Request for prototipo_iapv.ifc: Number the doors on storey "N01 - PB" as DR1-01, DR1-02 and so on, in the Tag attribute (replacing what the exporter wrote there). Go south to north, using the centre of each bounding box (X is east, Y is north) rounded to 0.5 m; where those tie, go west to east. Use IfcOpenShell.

First a look at what the model holds.

```python
import ifcopenshell
import ifcopenshell.util.element
import ifcopenshell.util.placement

model = ifcopenshell.open("prototipo_iapv.ifc")
print(model.schema)
storey = next(s for s in model.by_type("IfcBuildingStorey") if s.Name == "N01 - PB")
doors = [e for e in ifcopenshell.util.element.get_decomposition(storey) if e.is_a("IfcDoor")]
for e in sorted(doors, key=lambda e: e.id()):
    origin = ifcopenshell.util.placement.get_local_placement(e.ObjectPlacement)[:3, 3]
    print(e.id(), e.Tag, e.Name, origin.round(2) + 0.0, sep=" | ")
```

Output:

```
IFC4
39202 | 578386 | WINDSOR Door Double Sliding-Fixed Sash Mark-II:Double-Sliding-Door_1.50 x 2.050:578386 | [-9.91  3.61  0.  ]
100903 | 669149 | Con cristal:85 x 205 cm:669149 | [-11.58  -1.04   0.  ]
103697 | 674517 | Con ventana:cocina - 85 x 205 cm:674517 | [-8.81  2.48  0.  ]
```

```python
import ifcopenshell
import ifcopenshell.geom
import ifcopenshell.util.element
import ifcopenshell.util.shape

model = ifcopenshell.open("prototipo_iapv.ifc")
settings = ifcopenshell.geom.settings()
settings.set("use-world-coords", True)


def centre(element):
    shape = ifcopenshell.geom.create_shape(settings, element)
    return ifcopenshell.util.shape.get_bbox_centroid(shape.geometry)


storey = next(s for s in model.by_type("IfcBuildingStorey") if s.Name == "N01 - PB")
doors = [e for e in ifcopenshell.util.element.get_decomposition(storey) if e.is_a("IfcDoor")]

# Insertion points can sit at a corner or the storey origin, so sort by the geometry (in metres).
centres = {e: centre(e) for e in doors}
doors.sort(key=lambda e: (round(centres[e][1] / 0.5), centres[e][0]))

for i, e in enumerate(doors, start=1):
    number = f"DR1-{i:02d}"
    e.Tag = number
    print(e.id(), number)

model.write("prototipo_iapv_updated.ifc")
```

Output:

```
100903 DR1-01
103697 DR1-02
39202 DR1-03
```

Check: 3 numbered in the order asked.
